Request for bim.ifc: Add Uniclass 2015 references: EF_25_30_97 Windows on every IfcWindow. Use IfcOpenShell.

First a look at what the model holds.

```python
import ifcopenshell

model = ifcopenshell.open("bim.ifc")
print(model.schema)
print("classifications:", [c.Name for c in model.by_type("IfcClassification")])
for ifc_class in ("IfcDoor", "IfcRoof", "IfcStair", "IfcWall", "IfcWindow"):
    print(ifc_class, len(model.by_type(ifc_class)))
```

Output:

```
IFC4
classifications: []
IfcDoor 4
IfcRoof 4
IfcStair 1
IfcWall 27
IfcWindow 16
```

```python
import ifcopenshell
import ifcopenshell.api.classification

model = ifcopenshell.open("bim.ifc")

system = ifcopenshell.api.classification.add_classification(model, classification="Uniclass 2015")

codes = {
    "IfcWindow": ("EF_25_30_97", "Windows"),
}
for ifc_class, (code, name) in codes.items():
    products = model.by_type(ifc_class)
    ifcopenshell.api.classification.add_reference(
        model, products=products, classification=system, identification=code, name=name
    )
    print(code, len(products))

model.write("bim_rev.ifc")
```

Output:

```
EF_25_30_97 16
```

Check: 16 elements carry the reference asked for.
